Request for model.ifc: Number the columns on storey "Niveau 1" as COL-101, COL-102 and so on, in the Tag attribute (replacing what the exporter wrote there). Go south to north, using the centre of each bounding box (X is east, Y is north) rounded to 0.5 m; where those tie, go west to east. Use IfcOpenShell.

First a look at what the model holds.

```python
import ifcopenshell
import ifcopenshell.util.element
import ifcopenshell.util.placement

model = ifcopenshell.open("model.ifc")
print(model.schema)
storey = next(s for s in model.by_type("IfcBuildingStorey") if s.Name == "Niveau 1")
columns = [e for e in ifcopenshell.util.element.get_decomposition(storey) if e.is_a("IfcColumn")]
for e in sorted(columns, key=lambda e: e.id()):
    origin = ifcopenshell.util.placement.get_local_placement(e.ObjectPlacement)[:3, 3]
    print(e.id(), e.Tag, e.Name, origin.round(2) + 0.0, sep=" | ")
```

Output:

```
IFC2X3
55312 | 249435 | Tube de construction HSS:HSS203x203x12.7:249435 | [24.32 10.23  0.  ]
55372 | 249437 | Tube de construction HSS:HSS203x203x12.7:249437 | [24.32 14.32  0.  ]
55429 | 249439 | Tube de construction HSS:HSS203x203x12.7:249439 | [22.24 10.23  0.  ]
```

```python
import ifcopenshell
import ifcopenshell.geom
import ifcopenshell.util.element
import ifcopenshell.util.shape

model = ifcopenshell.open("model.ifc")
settings = ifcopenshell.geom.settings()
settings.set("use-world-coords", True)


def centre(element):
    shape = ifcopenshell.geom.create_shape(settings, element)
    return ifcopenshell.util.shape.get_bbox_centroid(shape.geometry)


storey = next(s for s in model.by_type("IfcBuildingStorey") if s.Name == "Niveau 1")
columns = [e for e in ifcopenshell.util.element.get_decomposition(storey) if e.is_a("IfcColumn")]

# Insertion points can sit at a corner or the storey origin, so sort by the geometry (in metres).
centres = {e: centre(e) for e in columns}
columns.sort(key=lambda e: (round(centres[e][1] / 0.5), centres[e][0]))

for i, e in enumerate(columns, start=1):
    number = f"COL-1{i:02d}"
    e.Tag = number
    print(e.id(), number)

model.write("model_v2.ifc")
```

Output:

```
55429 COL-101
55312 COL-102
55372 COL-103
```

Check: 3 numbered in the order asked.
